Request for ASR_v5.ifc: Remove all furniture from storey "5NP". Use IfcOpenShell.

First a look at what the model holds.

```python
import ifcopenshell
import ifcopenshell.util.element

model = ifcopenshell.open("ASR_v5.ifc")
print(model.schema)
storey = next(s for s in model.by_type("IfcBuildingStorey") if s.Name == "5NP")
furniture = [e for e in ifcopenshell.util.element.get_decomposition(storey) if e.is_a("IfcFurnishingElement")]
seen = {}
for e in furniture:
    element_type = ifcopenshell.util.element.get_type(e)
    name = element_type.Name if element_type not in (None, e) else None
    seen[name] = seen.get(name, 0) + 1
for name, count in sorted(seen.items(), key=str):
    print(count, "x", name)
```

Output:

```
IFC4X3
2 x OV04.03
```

```python
import ifcopenshell
import ifcopenshell.api.root
import ifcopenshell.util.element

model = ifcopenshell.open("ASR_v5.ifc")

storey = next(s for s in model.by_type("IfcBuildingStorey") if s.Name == "5NP")
furniture = [e for e in ifcopenshell.util.element.get_decomposition(storey) if e.is_a("IfcFurnishingElement")]

for e in furniture:
    ifcopenshell.api.root.remove_product(model, product=e)
print(len(furniture), "removed")

model.write("ASR_v5_v2.ifc")
```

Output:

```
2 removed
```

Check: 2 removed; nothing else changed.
